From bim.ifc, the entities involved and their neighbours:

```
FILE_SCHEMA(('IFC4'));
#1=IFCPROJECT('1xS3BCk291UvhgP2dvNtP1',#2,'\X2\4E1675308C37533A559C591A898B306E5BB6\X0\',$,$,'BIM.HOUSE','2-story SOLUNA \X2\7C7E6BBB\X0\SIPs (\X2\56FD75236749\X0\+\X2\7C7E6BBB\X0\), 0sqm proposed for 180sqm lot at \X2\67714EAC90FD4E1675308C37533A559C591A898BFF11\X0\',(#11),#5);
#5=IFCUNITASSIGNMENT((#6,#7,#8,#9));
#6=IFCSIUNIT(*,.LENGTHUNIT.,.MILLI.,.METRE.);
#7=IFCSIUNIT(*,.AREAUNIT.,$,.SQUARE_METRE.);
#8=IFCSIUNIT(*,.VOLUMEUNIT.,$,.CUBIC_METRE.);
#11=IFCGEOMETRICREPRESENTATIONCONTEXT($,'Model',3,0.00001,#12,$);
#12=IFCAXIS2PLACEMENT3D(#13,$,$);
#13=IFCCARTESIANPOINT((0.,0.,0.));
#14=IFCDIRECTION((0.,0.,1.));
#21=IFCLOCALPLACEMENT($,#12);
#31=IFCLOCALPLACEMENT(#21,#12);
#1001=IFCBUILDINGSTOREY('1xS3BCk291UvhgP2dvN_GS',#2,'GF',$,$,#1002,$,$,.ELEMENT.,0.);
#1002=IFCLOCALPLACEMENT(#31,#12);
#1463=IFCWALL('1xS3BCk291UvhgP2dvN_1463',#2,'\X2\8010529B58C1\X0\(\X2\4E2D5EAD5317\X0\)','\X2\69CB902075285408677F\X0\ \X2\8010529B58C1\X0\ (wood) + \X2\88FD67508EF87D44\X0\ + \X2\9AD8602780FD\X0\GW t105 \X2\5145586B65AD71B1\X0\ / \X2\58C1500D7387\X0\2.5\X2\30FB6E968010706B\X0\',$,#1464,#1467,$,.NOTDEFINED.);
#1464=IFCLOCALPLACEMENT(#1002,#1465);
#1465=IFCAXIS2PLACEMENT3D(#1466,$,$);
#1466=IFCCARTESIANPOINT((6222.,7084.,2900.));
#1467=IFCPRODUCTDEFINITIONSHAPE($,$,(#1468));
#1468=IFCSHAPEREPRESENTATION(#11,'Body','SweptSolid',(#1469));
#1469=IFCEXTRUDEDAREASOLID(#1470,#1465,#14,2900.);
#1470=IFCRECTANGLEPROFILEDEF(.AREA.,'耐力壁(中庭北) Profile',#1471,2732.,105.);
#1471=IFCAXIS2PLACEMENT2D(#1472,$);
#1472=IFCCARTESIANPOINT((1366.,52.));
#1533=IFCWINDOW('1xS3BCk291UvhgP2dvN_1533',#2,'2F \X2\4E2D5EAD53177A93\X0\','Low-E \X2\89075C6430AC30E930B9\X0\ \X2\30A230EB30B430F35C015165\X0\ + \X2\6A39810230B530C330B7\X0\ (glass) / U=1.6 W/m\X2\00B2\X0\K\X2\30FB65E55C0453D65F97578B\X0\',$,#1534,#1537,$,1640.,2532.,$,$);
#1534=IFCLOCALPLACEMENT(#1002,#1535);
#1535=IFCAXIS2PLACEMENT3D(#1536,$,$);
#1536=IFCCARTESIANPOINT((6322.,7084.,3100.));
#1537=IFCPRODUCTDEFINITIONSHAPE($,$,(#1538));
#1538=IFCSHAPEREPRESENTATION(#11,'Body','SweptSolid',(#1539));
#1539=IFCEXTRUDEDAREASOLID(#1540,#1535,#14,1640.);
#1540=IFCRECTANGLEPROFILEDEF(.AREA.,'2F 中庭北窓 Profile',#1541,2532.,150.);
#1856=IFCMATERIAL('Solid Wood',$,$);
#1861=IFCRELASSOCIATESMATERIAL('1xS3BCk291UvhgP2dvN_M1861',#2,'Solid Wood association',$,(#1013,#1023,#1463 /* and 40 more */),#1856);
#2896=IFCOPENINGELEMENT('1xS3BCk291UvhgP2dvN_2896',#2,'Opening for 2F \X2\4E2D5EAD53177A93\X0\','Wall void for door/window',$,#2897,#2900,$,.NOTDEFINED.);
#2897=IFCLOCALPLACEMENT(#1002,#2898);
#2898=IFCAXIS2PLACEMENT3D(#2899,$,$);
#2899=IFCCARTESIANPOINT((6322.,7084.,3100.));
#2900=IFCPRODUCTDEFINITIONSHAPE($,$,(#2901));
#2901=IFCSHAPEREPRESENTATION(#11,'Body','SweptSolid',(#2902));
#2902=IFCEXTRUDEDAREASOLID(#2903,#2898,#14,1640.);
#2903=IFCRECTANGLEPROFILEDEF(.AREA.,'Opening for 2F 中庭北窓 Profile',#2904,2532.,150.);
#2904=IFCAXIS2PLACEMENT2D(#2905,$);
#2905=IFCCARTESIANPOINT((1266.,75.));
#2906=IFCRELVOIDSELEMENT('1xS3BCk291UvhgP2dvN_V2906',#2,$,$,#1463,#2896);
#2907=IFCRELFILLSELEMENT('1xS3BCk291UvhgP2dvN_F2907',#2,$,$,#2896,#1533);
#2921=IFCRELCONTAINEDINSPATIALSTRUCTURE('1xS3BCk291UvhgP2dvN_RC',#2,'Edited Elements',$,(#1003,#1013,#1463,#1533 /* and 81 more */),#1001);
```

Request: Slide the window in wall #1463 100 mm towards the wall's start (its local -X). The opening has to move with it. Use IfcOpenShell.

```python
import ifcopenshell
import ifcopenshell.api.geometry
import ifcopenshell.util.placement
import ifcopenshell.util.unit

model = ifcopenshell.open("bim.ifc")
unit_scale = ifcopenshell.util.unit.calculate_unit_scale(model)

window = model.by_guid("1xS3BCk291UvhgP2dvN_1533")
opening = window.FillsVoids[0].RelatingOpeningElement
wall = opening.VoidsElements[0].RelatingBuildingElement

wall_matrix = ifcopenshell.util.placement.get_local_placement(wall.ObjectPlacement)
shift = wall_matrix[:3, 0] * -0.1 / unit_scale
before = ifcopenshell.util.placement.get_local_placement(window.ObjectPlacement)[:3, 3].copy()

# The window is not placed relative to its opening, so move both.
for product in (opening, window):
    matrix = ifcopenshell.util.placement.get_local_placement(product.ObjectPlacement)
    matrix[:3, 3] += shift
    ifcopenshell.api.geometry.edit_object_placement(model, product=product, matrix=matrix, is_si=False)

after = ifcopenshell.util.placement.get_local_placement(window.ObjectPlacement)[:3, 3]
print("window moved by", (after - before).round(3) + 0.0)

model.write("bim_v2.ifc")
```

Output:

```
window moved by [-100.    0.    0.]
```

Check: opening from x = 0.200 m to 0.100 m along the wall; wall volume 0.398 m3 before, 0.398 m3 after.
